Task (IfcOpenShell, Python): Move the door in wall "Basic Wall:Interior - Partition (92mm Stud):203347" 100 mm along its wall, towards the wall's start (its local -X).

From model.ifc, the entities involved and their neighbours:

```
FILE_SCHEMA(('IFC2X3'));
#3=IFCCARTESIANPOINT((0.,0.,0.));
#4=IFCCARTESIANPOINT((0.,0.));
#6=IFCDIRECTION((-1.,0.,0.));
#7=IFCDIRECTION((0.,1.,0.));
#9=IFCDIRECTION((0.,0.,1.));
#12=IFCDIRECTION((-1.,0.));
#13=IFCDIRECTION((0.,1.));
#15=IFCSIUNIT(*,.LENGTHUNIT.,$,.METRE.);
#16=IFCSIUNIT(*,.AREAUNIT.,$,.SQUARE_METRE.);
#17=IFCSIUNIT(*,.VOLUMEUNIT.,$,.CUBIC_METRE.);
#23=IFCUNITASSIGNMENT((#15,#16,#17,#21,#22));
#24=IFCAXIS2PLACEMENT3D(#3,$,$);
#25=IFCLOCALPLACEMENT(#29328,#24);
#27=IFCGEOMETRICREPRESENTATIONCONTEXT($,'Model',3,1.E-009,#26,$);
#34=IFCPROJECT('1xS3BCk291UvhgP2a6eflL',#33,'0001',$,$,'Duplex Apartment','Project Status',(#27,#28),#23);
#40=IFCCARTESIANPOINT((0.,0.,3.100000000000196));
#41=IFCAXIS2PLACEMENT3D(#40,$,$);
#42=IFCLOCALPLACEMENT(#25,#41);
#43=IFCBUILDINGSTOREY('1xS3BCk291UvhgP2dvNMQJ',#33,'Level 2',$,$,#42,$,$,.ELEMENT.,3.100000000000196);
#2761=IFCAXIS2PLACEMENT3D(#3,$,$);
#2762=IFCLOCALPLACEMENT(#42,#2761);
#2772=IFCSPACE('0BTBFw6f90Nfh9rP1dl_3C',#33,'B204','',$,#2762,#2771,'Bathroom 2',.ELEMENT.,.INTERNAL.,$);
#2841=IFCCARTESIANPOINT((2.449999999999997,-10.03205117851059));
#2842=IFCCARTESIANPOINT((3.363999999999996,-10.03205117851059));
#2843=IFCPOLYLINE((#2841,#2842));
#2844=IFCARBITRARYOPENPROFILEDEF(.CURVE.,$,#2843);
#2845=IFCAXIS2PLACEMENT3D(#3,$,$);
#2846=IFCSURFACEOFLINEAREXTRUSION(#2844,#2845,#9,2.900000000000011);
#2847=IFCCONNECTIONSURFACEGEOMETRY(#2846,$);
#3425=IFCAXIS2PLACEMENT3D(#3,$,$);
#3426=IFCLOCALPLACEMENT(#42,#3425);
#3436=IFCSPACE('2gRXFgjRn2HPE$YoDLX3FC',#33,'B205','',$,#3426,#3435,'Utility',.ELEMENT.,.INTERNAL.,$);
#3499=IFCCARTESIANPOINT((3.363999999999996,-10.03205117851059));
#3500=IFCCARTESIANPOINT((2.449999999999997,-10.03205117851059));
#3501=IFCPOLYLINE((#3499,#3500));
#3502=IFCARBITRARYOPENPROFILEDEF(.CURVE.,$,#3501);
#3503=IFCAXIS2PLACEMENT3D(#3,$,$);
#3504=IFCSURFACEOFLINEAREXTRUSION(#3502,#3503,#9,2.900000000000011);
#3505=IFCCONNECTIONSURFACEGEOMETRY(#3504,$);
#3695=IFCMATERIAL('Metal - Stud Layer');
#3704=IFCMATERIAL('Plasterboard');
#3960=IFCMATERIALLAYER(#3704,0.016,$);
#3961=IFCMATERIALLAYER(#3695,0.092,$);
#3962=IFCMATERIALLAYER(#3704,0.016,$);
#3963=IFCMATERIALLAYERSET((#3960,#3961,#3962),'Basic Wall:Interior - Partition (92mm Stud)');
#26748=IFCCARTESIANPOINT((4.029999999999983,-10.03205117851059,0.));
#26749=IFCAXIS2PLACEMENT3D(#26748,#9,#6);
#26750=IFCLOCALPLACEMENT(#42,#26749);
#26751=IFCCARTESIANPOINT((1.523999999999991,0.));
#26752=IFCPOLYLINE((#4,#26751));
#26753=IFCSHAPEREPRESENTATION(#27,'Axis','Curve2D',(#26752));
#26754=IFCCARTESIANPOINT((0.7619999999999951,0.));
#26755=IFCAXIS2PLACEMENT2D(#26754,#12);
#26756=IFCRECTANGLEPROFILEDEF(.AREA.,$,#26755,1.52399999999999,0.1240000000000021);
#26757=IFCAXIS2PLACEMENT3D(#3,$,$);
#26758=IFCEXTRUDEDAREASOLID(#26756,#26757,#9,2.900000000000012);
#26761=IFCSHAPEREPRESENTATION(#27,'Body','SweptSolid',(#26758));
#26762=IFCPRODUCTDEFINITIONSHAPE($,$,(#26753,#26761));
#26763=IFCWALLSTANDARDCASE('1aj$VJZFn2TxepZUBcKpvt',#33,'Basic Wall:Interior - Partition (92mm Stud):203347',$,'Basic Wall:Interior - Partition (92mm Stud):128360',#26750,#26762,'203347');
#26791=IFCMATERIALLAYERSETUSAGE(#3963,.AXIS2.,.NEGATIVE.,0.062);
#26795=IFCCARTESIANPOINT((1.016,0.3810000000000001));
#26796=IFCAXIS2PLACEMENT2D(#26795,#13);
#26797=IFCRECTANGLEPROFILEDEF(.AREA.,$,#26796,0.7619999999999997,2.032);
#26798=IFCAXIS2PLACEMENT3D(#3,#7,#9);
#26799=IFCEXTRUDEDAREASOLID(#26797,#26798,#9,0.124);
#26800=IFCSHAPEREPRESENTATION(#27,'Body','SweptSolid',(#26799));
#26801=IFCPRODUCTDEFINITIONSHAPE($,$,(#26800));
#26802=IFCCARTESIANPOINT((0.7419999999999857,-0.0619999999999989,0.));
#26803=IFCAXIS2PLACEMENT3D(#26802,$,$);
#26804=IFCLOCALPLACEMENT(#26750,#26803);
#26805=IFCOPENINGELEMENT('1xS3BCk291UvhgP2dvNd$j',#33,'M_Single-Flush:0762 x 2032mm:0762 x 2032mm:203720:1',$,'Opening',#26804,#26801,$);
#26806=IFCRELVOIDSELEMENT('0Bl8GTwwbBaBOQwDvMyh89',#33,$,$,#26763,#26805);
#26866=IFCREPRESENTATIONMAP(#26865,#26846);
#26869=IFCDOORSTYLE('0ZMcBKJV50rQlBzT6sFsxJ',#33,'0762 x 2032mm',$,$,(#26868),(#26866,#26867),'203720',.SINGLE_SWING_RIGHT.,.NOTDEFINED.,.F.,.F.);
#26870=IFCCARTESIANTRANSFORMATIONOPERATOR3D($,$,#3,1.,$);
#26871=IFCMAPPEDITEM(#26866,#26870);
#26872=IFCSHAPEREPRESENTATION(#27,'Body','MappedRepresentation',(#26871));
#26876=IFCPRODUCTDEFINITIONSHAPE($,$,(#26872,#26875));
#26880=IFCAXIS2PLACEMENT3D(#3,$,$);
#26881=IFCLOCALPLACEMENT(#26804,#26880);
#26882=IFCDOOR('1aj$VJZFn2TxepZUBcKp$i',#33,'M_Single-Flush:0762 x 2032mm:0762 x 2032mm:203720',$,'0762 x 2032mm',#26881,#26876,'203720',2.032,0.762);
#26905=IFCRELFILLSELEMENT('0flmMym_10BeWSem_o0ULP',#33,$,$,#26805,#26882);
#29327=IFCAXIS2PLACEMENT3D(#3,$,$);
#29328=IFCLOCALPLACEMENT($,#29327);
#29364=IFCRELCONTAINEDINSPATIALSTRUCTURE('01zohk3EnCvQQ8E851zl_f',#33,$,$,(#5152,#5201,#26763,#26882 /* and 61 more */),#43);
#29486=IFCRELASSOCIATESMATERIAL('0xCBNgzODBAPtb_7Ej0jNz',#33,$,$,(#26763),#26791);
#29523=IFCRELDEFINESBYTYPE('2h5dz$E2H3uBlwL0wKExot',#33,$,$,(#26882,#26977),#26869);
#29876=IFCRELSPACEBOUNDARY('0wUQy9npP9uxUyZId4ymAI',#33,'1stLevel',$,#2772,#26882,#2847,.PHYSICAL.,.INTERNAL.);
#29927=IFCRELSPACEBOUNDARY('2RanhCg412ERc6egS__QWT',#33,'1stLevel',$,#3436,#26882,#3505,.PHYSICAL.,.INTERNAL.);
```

```python
import numpy as np
import ifcopenshell
import ifcopenshell.api.geometry
import ifcopenshell.util.placement
import ifcopenshell.util.unit

model = ifcopenshell.open("model.ifc")
unit_scale = ifcopenshell.util.unit.calculate_unit_scale(model)

door = model.by_guid("1aj$VJZFn2TxepZUBcKp$i")
opening = door.FillsVoids[0].RelatingOpeningElement
wall = opening.VoidsElements[0].RelatingBuildingElement

wall_matrix = ifcopenshell.util.placement.get_local_placement(wall.ObjectPlacement)
shift = wall_matrix[:3, 0] * -0.1 / unit_scale
before = ifcopenshell.util.placement.get_local_placement(door.ObjectPlacement)[:3, 3].copy()

# The door is placed relative to its opening, so it follows when the opening moves.
matrix = ifcopenshell.util.placement.get_local_placement(opening.ObjectPlacement)
matrix[:3, 3] += shift
ifcopenshell.api.geometry.edit_object_placement(
    model, product=opening, matrix=matrix, is_si=False, should_transform_children=True
)

# Space boundary surfaces are stored in each space's coordinates; move them too.
for rel in door.ProvidesBoundaries:
    if not rel.ConnectionGeometry:
        continue
    surface = rel.ConnectionGeometry.SurfaceOnRelatingElement
    space_matrix = ifcopenshell.util.placement.get_local_placement(rel.RelatingSpace.ObjectPlacement)
    point = np.array(surface.Position.Location.Coordinates) + space_matrix[:3, :3].T @ shift
    surface.Position = model.createIfcAxis2Placement3D(
        model.createIfcCartesianPoint(point.tolist()), surface.Position.Axis, surface.Position.RefDirection
    )

after = ifcopenshell.util.placement.get_local_placement(door.ObjectPlacement)[:3, 3]
print("door moved by", (after - before).round(3) + 0.0)

model.write("model_updated.ifc")
```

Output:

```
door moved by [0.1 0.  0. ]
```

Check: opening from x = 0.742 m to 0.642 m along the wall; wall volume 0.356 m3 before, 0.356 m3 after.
